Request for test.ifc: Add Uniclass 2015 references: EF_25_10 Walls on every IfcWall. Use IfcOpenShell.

First a look at what the model holds.

```python
import ifcopenshell

model = ifcopenshell.open("test.ifc")
print(model.schema)
print("classifications:", [c.Name for c in model.by_type("IfcClassification")])
for ifc_class in ("IfcDoor", "IfcRoof", "IfcStair", "IfcWall", "IfcWindow"):
    print(ifc_class, len(model.by_type(ifc_class)))
```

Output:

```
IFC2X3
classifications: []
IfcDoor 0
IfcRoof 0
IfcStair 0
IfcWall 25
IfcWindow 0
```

```python
import ifcopenshell
import ifcopenshell.api.classification

model = ifcopenshell.open("test.ifc")

# IFC2X3 requires Source and Edition and has no link from the project to the system.
system = model.create_entity("IfcClassification", Source="NBS", Edition="2015", Name="Uniclass 2015")

codes = {
    "IfcWall": ("EF_25_10", "Walls"),
}
for ifc_class, (code, name) in codes.items():
    products = model.by_type(ifc_class)
    ifcopenshell.api.classification.add_reference(
        model, products=products, classification=system, identification=code, name=name
    )
    print(code, len(products))

model.write("test_v2.ifc")
```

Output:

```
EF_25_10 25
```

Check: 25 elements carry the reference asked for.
